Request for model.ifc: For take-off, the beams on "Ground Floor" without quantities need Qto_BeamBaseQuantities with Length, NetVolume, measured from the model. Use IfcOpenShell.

First a look at what the model holds.

```python
import ifcopenshell
import ifcopenshell.util.element
import ifcopenshell.util.unit

model = ifcopenshell.open("model.ifc")
print(model.schema)
for unit_type in ("LENGTHUNIT", "AREAUNIT", "VOLUMEUNIT"):
    print(unit_type, ifcopenshell.util.unit.calculate_unit_scale(model, unit_type))
storey = next(s for s in model.by_type("IfcBuildingStorey") if s.Name == "Ground Floor")
beams = [e for e in ifcopenshell.util.element.get_decomposition(storey) if e.is_a("IfcBeam")]
for e in sorted(beams, key=lambda e: e.id()):
    print(e.id(), e.is_a(), e.Name, list(ifcopenshell.util.element.get_psets(e, qtos_only=True)), sep=" | ")
```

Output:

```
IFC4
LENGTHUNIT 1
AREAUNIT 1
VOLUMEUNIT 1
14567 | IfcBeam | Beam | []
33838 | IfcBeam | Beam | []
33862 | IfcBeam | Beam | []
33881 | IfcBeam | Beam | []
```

```python
import ifcopenshell
import ifcopenshell.api.pset
import ifcopenshell.geom
import ifcopenshell.util.element
import ifcopenshell.util.shape
import ifcopenshell.util.unit

model = ifcopenshell.open("model.ifc")
unit_scale = ifcopenshell.util.unit.calculate_unit_scale(model)
volume_scale = ifcopenshell.util.unit.calculate_unit_scale(model, "VOLUMEUNIT")
settings = ifcopenshell.geom.settings()

storey = next(s for s in model.by_type("IfcBuildingStorey") if s.Name == "Ground Floor")
beams = [e for e in ifcopenshell.util.element.get_decomposition(storey) if e.is_a("IfcBeam")]

for e in sorted(beams, key=lambda e: e.id()):
    if ifcopenshell.util.element.get_psets(e, qtos_only=True, should_inherit=False):
        continue
    # Geometry comes back in metres, in the element's own axes.
    shape = ifcopenshell.geom.create_shape(settings, e)
    values = {
        "Length": ifcopenshell.util.shape.get_max_xyz(shape.geometry) / unit_scale,
        "NetVolume": ifcopenshell.util.shape.get_volume(shape.geometry) / volume_scale,
    }
    qto = ifcopenshell.api.pset.add_qto(model, product=e, name="Qto_BeamBaseQuantities")
    ifcopenshell.api.pset.edit_qto(model, qto=qto, properties=values)
    print(e.id(), {k: round(v, 3) for k, v in values.items()})

model.write("model_rev.ifc")
```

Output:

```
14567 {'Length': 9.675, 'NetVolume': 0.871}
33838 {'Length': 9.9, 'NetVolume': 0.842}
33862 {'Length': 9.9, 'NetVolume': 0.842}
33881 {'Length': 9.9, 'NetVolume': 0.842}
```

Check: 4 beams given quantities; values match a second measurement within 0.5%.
